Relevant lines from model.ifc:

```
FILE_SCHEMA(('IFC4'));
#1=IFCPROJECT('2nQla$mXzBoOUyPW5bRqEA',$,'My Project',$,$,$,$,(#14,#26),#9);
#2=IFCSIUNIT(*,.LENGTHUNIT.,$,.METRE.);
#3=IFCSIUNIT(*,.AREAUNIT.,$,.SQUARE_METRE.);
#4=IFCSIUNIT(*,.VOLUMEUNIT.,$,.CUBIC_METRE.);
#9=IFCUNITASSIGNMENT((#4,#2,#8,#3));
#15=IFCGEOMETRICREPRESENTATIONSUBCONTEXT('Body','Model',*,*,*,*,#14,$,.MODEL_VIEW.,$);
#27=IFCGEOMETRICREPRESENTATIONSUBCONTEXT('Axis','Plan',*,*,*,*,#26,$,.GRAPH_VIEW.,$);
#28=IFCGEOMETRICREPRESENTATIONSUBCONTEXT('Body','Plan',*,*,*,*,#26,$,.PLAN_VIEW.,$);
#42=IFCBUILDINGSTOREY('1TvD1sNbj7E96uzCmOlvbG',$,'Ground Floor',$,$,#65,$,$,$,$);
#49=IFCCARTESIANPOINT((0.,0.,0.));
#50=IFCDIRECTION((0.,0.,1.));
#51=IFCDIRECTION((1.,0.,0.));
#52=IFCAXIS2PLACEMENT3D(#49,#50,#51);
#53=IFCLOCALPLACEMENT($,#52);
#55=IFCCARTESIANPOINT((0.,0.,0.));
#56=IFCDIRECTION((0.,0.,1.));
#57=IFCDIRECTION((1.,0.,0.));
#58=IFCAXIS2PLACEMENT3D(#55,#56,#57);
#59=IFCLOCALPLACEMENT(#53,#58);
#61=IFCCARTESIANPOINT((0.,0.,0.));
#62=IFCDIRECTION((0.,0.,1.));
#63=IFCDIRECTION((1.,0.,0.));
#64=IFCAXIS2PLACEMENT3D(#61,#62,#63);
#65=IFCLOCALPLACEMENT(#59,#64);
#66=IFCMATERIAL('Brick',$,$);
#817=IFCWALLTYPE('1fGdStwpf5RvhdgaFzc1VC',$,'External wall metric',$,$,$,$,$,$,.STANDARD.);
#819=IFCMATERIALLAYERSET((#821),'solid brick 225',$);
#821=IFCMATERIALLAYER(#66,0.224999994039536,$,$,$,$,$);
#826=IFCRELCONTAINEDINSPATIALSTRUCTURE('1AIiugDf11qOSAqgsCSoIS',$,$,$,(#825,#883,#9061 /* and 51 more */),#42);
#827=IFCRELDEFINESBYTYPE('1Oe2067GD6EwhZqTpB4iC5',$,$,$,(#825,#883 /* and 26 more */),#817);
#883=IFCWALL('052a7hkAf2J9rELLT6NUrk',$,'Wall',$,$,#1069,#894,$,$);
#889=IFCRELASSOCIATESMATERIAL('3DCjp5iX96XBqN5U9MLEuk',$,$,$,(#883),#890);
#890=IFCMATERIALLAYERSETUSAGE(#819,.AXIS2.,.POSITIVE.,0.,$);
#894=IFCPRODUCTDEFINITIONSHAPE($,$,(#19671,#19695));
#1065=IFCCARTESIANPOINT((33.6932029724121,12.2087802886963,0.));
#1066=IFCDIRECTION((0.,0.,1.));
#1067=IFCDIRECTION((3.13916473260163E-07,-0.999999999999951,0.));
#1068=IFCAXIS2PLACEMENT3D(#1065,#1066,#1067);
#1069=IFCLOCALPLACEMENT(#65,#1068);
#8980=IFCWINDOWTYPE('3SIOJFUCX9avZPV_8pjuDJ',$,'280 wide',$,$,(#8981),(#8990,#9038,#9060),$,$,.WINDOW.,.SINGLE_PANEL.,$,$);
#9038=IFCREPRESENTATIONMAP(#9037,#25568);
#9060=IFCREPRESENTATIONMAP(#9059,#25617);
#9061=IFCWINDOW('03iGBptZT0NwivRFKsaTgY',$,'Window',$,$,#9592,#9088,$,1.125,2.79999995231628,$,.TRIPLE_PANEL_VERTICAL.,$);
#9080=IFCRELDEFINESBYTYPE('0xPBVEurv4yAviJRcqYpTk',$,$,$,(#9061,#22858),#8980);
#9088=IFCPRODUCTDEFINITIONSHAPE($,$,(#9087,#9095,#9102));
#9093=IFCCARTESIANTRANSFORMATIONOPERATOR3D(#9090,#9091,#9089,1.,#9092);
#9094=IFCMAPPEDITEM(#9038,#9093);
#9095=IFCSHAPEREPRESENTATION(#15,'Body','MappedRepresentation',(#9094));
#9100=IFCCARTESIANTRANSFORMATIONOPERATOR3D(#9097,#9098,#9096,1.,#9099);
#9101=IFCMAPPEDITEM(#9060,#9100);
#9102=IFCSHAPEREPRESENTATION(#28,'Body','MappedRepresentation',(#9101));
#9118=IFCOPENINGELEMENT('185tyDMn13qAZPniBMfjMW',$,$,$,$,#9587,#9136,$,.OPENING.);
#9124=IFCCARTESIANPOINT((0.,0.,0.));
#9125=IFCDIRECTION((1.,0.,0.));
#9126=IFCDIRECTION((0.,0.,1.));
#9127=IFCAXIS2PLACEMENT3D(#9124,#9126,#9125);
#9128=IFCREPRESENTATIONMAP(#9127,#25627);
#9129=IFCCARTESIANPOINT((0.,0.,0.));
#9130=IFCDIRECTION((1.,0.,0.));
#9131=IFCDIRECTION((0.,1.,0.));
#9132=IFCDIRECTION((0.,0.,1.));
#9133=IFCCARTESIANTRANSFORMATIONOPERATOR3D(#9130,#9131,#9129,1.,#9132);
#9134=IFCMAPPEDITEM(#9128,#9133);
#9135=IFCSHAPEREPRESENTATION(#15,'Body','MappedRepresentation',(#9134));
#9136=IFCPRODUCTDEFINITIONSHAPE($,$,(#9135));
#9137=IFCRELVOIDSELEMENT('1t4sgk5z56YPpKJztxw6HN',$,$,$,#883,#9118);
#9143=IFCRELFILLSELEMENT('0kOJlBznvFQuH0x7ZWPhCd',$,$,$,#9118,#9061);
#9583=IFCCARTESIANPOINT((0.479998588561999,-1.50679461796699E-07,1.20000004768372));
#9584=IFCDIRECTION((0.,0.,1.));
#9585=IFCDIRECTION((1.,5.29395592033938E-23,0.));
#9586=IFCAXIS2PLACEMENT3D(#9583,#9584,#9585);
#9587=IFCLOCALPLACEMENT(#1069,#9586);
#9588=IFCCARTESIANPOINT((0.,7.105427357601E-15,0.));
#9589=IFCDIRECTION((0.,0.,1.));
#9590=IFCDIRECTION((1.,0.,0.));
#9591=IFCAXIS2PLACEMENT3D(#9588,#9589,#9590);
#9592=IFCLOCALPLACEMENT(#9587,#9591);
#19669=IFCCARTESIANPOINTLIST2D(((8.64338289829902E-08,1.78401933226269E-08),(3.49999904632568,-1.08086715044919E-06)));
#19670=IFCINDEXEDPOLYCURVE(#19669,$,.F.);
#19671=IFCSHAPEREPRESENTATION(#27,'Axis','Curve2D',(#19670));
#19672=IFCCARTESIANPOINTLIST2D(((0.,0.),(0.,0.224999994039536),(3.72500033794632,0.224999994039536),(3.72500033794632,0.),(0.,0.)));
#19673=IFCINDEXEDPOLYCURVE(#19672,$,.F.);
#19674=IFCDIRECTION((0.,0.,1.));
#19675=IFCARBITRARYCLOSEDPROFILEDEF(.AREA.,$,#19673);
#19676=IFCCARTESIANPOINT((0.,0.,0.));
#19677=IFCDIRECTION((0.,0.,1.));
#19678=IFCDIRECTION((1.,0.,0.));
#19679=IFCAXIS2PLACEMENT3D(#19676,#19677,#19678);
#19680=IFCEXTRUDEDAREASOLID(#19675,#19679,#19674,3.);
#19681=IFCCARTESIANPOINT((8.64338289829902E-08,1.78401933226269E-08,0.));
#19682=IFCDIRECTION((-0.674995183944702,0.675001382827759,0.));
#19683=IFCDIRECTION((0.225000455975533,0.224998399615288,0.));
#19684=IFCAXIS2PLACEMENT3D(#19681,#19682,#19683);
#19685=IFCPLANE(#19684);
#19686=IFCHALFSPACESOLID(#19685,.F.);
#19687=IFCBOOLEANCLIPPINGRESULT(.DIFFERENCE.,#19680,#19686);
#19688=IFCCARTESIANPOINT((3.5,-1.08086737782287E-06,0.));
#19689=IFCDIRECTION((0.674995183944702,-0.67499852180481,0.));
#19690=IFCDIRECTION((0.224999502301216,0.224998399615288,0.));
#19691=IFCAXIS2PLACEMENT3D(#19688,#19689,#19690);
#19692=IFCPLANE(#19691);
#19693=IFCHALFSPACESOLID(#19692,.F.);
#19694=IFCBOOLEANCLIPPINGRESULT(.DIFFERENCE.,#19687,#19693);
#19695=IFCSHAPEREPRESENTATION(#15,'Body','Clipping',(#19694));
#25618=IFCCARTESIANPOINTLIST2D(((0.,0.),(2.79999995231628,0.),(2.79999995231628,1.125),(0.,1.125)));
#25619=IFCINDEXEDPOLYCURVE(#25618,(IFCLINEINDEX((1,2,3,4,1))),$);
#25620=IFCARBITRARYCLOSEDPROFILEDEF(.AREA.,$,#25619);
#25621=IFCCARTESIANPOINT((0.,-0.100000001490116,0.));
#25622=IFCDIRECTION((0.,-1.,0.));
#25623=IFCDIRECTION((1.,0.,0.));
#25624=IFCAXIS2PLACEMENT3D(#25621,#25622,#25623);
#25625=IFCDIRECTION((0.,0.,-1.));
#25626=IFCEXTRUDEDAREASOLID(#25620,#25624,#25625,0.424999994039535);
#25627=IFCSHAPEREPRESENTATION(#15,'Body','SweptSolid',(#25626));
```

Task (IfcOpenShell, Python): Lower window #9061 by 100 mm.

```python
import numpy as np
import ifcopenshell
import ifcopenshell.api.geometry
import ifcopenshell.util.placement
import ifcopenshell.util.unit

model = ifcopenshell.open("model.ifc")
unit_scale = ifcopenshell.util.unit.calculate_unit_scale(model)

window = model.by_id(9061)
opening = window.FillsVoids[0].RelatingOpeningElement
dz = -0.1 / unit_scale

shift = np.array([0.0, 0.0, dz])
# The window is placed relative to its opening, so it follows when the opening moves.
matrix = ifcopenshell.util.placement.get_local_placement(opening.ObjectPlacement)
matrix[:3, 3] += shift
ifcopenshell.api.geometry.edit_object_placement(
    model, product=opening, matrix=matrix, is_si=False, should_transform_children=True
)

print(f"moved by {dz * unit_scale:+.3f} m")

model.write("model-out.ifc")
```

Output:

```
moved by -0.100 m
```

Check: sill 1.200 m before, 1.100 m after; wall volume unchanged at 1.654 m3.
